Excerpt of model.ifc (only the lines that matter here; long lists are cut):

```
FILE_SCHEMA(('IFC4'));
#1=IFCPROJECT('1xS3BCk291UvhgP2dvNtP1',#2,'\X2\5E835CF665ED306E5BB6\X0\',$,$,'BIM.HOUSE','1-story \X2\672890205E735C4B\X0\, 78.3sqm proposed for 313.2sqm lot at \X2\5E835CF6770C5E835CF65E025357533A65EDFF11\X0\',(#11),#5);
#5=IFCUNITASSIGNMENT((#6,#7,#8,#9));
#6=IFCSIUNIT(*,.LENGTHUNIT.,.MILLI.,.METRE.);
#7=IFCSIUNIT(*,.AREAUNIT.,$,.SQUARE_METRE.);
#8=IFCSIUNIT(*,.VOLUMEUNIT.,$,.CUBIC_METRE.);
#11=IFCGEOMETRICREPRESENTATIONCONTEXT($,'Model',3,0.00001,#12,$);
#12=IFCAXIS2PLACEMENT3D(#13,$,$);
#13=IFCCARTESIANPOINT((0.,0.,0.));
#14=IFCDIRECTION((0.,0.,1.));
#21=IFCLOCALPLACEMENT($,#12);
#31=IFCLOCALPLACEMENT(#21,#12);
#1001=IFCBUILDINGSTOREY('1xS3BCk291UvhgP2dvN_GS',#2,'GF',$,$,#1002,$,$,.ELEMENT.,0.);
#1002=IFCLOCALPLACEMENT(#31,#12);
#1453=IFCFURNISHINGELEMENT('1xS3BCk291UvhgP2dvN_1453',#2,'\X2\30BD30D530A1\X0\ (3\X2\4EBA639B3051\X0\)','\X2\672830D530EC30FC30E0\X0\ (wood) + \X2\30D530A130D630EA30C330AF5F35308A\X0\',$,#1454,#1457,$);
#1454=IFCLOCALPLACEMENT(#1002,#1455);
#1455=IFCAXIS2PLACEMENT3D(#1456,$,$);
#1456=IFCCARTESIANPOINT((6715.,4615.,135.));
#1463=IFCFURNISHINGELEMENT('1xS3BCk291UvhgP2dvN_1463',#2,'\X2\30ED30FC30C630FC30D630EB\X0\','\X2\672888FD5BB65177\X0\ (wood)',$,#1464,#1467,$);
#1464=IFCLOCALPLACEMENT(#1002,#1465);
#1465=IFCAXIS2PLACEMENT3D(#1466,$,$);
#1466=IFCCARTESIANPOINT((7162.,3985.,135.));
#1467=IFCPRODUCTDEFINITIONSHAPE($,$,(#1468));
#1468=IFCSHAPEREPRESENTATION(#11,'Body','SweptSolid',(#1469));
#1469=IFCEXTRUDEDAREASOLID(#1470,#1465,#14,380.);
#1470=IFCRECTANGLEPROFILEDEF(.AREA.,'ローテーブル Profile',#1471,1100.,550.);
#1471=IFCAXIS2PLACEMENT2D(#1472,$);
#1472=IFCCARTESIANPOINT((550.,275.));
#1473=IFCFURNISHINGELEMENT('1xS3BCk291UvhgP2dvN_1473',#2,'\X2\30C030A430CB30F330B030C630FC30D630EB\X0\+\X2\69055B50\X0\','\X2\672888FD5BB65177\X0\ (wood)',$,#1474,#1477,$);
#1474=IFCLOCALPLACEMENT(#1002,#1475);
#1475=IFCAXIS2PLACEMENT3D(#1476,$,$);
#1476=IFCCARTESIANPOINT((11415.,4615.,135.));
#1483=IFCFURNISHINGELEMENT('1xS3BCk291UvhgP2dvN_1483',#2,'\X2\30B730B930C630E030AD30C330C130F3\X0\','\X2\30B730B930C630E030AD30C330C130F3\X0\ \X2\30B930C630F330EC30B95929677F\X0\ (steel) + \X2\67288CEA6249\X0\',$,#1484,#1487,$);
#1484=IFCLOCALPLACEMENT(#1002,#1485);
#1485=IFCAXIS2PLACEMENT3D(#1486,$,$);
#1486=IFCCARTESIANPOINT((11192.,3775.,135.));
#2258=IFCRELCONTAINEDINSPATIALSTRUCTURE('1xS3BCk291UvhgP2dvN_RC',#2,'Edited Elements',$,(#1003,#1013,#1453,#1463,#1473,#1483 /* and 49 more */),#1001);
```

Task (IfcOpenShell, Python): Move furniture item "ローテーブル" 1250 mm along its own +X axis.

```python
import ifcopenshell
import ifcopenshell.api.geometry
import ifcopenshell.util.placement
import ifcopenshell.util.unit

model = ifcopenshell.open("model.ifc")
unit_scale = ifcopenshell.util.unit.calculate_unit_scale(model)

item = model.by_id(1463)
matrix = ifcopenshell.util.placement.get_local_placement(item.ObjectPlacement)
matrix[:3, 3] += matrix[:3, 0] * 1.25 / unit_scale
ifcopenshell.api.geometry.edit_object_placement(model, product=item, matrix=matrix, is_si=False)

print(ifcopenshell.util.placement.get_local_placement(item.ObjectPlacement).round(3) + 0.0)

model.write("model-out.ifc")
```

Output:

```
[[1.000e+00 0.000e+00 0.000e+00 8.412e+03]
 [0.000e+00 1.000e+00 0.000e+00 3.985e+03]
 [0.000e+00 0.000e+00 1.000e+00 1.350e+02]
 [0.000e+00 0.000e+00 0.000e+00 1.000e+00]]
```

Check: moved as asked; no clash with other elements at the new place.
